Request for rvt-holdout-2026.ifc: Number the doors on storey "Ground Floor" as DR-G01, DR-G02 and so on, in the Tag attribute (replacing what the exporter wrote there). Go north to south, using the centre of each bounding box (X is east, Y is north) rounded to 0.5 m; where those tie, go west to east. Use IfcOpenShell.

First a look at what the model holds.

```python
import ifcopenshell
import ifcopenshell.util.element
import ifcopenshell.util.placement

model = ifcopenshell.open("rvt-holdout-2026.ifc")
print(model.schema)
storey = next(s for s in model.by_type("IfcBuildingStorey") if s.Name == "Ground Floor")
doors = [e for e in ifcopenshell.util.element.get_decomposition(storey) if e.is_a("IfcDoor")]
for e in sorted(doors, key=lambda e: e.id()):
    origin = ifcopenshell.util.placement.get_local_placement(e.ObjectPlacement)[:3, 3]
    print(e.id(), e.Tag, e.Name, origin.round(2) + 0.0, sep=" | ")
```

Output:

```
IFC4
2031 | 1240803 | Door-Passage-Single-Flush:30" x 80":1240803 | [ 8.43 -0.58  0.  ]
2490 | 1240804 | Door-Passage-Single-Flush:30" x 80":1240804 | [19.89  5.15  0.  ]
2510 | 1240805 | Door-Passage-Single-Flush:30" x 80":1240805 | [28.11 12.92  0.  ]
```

```python
import ifcopenshell
import ifcopenshell.geom
import ifcopenshell.util.element
import ifcopenshell.util.shape

model = ifcopenshell.open("rvt-holdout-2026.ifc")
settings = ifcopenshell.geom.settings()
settings.set("use-world-coords", True)


def centre(element):
    shape = ifcopenshell.geom.create_shape(settings, element)
    return ifcopenshell.util.shape.get_bbox_centroid(shape.geometry)


storey = next(s for s in model.by_type("IfcBuildingStorey") if s.Name == "Ground Floor")
doors = [e for e in ifcopenshell.util.element.get_decomposition(storey) if e.is_a("IfcDoor")]

# Insertion points can sit at a corner or the storey origin, so sort by the geometry (in metres).
centres = {e: centre(e) for e in doors}
doors.sort(key=lambda e: (-round(centres[e][1] / 0.5), centres[e][0]))

for i, e in enumerate(doors, start=1):
    number = f"DR-G{i:02d}"
    e.Tag = number
    print(e.id(), number)

model.write("rvt-holdout-2026_v2.ifc")
```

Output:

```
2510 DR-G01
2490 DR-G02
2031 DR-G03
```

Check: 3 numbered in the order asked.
